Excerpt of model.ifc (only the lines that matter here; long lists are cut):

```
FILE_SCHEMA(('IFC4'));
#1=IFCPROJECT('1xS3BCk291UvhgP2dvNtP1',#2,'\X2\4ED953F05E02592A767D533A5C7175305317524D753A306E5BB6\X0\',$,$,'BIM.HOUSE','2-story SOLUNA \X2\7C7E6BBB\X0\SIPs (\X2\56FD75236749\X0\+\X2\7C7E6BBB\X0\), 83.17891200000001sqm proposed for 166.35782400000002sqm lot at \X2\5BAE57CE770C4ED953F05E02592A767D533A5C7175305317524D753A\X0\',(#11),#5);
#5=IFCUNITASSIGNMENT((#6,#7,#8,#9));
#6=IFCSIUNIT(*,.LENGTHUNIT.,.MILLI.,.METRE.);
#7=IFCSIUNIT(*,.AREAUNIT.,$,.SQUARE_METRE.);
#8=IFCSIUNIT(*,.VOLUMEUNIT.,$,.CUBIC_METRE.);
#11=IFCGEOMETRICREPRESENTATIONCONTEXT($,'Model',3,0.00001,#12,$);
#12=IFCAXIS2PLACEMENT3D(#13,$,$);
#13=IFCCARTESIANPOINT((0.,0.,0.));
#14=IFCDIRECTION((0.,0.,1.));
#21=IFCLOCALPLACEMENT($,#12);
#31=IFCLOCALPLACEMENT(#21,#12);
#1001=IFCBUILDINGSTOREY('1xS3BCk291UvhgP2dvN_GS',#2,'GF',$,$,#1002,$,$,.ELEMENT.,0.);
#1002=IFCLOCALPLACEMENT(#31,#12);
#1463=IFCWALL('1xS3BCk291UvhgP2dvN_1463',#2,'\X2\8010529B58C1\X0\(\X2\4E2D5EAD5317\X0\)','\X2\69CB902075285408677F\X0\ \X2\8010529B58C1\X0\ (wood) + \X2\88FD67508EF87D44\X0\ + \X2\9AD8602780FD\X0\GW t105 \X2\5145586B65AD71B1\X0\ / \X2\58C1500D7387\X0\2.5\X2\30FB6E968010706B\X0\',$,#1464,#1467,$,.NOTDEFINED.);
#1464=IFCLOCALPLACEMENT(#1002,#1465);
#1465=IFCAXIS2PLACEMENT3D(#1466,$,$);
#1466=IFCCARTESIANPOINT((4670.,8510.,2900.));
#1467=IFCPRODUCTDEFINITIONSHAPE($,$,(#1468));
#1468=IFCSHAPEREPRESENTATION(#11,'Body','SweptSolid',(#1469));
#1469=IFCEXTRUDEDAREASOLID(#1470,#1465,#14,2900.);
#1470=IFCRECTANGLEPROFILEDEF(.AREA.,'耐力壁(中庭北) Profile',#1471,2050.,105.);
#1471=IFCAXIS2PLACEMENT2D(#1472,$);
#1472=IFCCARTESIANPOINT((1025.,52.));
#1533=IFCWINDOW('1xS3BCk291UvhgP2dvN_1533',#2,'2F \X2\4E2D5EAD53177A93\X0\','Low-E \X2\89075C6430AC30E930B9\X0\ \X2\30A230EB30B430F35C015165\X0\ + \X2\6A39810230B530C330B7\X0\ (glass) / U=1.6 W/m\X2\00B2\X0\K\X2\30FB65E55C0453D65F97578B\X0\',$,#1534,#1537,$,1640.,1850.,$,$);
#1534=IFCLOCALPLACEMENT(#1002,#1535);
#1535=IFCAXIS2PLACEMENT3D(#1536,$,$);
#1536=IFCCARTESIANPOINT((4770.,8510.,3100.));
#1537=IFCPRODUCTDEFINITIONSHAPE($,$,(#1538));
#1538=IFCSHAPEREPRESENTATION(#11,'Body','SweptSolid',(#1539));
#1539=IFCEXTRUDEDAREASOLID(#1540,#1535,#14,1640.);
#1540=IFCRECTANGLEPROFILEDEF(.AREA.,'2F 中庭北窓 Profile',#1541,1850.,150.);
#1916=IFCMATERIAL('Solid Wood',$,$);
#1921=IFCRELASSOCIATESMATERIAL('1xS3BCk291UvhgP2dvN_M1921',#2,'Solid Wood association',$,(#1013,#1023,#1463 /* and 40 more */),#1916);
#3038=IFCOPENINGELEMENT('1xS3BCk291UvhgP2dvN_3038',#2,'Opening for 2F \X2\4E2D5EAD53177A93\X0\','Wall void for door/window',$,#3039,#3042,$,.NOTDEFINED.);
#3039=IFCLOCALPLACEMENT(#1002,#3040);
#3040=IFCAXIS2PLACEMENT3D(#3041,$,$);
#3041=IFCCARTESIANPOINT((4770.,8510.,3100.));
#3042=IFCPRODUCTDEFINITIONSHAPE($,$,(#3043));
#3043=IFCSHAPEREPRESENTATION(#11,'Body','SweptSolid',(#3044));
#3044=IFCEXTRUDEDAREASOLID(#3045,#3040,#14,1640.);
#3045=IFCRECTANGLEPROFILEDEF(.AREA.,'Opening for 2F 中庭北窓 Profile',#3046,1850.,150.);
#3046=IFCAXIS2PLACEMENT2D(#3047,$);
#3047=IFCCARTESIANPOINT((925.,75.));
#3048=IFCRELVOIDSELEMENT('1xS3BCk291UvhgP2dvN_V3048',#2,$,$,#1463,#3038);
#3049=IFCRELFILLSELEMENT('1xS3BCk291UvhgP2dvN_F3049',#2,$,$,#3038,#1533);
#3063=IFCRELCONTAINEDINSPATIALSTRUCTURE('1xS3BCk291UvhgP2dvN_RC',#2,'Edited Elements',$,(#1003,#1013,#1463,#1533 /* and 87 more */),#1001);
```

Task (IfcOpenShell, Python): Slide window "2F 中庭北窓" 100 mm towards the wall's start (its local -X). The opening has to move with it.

```python
import ifcopenshell
import ifcopenshell.api.geometry
import ifcopenshell.util.placement
import ifcopenshell.util.unit

model = ifcopenshell.open("model.ifc")
unit_scale = ifcopenshell.util.unit.calculate_unit_scale(model)

window = model.by_id(1533)
opening = window.FillsVoids[0].RelatingOpeningElement
wall = opening.VoidsElements[0].RelatingBuildingElement

wall_matrix = ifcopenshell.util.placement.get_local_placement(wall.ObjectPlacement)
shift = wall_matrix[:3, 0] * -0.1 / unit_scale
before = ifcopenshell.util.placement.get_local_placement(window.ObjectPlacement)[:3, 3].copy()

# The window is not placed relative to its opening, so move both.
for product in (opening, window):
    matrix = ifcopenshell.util.placement.get_local_placement(product.ObjectPlacement)
    matrix[:3, 3] += shift
    ifcopenshell.api.geometry.edit_object_placement(model, product=product, matrix=matrix, is_si=False)

after = ifcopenshell.util.placement.get_local_placement(window.ObjectPlacement)[:3, 3]
print("window moved by", (after - before).round(3) + 0.0)

model.write("model_rev.ifc")
```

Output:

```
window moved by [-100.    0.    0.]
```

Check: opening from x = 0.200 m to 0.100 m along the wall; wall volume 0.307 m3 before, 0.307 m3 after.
